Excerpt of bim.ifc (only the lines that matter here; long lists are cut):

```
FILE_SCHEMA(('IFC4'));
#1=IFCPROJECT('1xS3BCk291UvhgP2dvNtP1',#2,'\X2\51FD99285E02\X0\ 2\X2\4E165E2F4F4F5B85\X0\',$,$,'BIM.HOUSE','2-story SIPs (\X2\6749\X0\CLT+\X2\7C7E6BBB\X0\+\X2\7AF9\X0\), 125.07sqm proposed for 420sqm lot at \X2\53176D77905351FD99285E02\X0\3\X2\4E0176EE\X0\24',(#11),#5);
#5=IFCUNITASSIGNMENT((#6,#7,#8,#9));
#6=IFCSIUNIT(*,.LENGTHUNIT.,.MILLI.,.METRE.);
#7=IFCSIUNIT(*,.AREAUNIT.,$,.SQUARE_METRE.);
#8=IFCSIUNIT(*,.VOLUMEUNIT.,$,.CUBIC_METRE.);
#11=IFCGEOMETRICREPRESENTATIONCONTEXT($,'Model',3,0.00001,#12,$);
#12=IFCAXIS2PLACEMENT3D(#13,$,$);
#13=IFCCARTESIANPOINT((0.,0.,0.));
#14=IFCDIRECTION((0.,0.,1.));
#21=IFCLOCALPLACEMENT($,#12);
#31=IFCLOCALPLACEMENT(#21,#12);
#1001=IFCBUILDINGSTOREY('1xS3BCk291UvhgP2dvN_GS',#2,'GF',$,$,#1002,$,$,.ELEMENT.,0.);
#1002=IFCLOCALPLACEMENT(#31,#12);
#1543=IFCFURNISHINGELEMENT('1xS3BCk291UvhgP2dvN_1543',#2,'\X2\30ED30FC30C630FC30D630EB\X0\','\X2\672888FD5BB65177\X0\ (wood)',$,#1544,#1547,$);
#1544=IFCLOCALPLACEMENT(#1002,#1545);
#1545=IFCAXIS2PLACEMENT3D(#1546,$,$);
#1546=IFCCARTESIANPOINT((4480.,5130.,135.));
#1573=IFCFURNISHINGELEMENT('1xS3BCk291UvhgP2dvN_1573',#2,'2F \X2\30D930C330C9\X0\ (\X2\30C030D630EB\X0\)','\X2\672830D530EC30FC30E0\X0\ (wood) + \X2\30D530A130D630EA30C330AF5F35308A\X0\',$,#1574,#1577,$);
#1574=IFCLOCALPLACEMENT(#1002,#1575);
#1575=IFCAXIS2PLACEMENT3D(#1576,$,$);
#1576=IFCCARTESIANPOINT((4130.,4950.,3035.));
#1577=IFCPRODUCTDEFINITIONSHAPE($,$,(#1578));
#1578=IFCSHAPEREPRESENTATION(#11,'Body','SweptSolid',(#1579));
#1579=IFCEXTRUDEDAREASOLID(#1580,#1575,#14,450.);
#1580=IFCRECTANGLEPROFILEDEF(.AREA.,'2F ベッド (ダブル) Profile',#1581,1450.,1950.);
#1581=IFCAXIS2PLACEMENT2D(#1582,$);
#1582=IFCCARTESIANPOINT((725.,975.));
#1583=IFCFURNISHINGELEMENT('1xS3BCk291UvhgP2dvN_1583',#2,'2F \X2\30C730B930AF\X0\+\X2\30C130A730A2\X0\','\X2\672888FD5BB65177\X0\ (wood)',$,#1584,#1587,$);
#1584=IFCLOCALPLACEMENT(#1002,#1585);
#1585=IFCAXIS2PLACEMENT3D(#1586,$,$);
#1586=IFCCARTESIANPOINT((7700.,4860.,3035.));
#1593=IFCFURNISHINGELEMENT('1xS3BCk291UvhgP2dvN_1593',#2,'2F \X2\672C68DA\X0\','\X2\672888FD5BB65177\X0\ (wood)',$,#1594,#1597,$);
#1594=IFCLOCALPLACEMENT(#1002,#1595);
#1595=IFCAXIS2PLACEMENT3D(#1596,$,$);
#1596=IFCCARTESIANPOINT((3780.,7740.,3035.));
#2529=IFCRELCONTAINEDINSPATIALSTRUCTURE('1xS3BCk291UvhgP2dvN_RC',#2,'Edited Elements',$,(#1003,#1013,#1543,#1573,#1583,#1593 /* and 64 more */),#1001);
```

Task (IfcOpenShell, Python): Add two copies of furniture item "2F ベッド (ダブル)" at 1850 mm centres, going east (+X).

```python
import numpy as np
import ifcopenshell
import ifcopenshell.api.geometry
import ifcopenshell.api.root
import ifcopenshell.util.element
import ifcopenshell.util.placement

model = ifcopenshell.open("bim.ifc")


def reuse_history(source, copy):
    """copy_class also copies each property set's owner history, people and application; keep the originals."""
    for rel in copy.IsDefinedBy:
        if rel.is_a("IfcRelDefinesByProperties") and (history := rel.RelatingPropertyDefinition.OwnerHistory):
            rel.RelatingPropertyDefinition.OwnerHistory = source.OwnerHistory
            ifcopenshell.util.element.remove_deep2(model, history)


source = model.by_id(1573)
base = ifcopenshell.util.placement.get_local_placement(source.ObjectPlacement)
step = np.array([1.0, 0.0, 0.0]) * 1850.0

for i in range(1, 3):
    copy = ifcopenshell.api.root.copy_class(model, product=source)
    copy.Representation = ifcopenshell.util.element.copy_deep(
        model, source.Representation, exclude=["IfcGeometricRepresentationContext", "IfcRepresentationMap"]
    )
    reuse_history(source, copy)
    matrix = base.copy()
    matrix[:3, 3] += i * step
    print("added at", matrix[:3, 3].round(3) + 0.0)
    ifcopenshell.api.geometry.edit_object_placement(model, product=copy, matrix=matrix, is_si=False)

model.write("bim-out.ifc")
```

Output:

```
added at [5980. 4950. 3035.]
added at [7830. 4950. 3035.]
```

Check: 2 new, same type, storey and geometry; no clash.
